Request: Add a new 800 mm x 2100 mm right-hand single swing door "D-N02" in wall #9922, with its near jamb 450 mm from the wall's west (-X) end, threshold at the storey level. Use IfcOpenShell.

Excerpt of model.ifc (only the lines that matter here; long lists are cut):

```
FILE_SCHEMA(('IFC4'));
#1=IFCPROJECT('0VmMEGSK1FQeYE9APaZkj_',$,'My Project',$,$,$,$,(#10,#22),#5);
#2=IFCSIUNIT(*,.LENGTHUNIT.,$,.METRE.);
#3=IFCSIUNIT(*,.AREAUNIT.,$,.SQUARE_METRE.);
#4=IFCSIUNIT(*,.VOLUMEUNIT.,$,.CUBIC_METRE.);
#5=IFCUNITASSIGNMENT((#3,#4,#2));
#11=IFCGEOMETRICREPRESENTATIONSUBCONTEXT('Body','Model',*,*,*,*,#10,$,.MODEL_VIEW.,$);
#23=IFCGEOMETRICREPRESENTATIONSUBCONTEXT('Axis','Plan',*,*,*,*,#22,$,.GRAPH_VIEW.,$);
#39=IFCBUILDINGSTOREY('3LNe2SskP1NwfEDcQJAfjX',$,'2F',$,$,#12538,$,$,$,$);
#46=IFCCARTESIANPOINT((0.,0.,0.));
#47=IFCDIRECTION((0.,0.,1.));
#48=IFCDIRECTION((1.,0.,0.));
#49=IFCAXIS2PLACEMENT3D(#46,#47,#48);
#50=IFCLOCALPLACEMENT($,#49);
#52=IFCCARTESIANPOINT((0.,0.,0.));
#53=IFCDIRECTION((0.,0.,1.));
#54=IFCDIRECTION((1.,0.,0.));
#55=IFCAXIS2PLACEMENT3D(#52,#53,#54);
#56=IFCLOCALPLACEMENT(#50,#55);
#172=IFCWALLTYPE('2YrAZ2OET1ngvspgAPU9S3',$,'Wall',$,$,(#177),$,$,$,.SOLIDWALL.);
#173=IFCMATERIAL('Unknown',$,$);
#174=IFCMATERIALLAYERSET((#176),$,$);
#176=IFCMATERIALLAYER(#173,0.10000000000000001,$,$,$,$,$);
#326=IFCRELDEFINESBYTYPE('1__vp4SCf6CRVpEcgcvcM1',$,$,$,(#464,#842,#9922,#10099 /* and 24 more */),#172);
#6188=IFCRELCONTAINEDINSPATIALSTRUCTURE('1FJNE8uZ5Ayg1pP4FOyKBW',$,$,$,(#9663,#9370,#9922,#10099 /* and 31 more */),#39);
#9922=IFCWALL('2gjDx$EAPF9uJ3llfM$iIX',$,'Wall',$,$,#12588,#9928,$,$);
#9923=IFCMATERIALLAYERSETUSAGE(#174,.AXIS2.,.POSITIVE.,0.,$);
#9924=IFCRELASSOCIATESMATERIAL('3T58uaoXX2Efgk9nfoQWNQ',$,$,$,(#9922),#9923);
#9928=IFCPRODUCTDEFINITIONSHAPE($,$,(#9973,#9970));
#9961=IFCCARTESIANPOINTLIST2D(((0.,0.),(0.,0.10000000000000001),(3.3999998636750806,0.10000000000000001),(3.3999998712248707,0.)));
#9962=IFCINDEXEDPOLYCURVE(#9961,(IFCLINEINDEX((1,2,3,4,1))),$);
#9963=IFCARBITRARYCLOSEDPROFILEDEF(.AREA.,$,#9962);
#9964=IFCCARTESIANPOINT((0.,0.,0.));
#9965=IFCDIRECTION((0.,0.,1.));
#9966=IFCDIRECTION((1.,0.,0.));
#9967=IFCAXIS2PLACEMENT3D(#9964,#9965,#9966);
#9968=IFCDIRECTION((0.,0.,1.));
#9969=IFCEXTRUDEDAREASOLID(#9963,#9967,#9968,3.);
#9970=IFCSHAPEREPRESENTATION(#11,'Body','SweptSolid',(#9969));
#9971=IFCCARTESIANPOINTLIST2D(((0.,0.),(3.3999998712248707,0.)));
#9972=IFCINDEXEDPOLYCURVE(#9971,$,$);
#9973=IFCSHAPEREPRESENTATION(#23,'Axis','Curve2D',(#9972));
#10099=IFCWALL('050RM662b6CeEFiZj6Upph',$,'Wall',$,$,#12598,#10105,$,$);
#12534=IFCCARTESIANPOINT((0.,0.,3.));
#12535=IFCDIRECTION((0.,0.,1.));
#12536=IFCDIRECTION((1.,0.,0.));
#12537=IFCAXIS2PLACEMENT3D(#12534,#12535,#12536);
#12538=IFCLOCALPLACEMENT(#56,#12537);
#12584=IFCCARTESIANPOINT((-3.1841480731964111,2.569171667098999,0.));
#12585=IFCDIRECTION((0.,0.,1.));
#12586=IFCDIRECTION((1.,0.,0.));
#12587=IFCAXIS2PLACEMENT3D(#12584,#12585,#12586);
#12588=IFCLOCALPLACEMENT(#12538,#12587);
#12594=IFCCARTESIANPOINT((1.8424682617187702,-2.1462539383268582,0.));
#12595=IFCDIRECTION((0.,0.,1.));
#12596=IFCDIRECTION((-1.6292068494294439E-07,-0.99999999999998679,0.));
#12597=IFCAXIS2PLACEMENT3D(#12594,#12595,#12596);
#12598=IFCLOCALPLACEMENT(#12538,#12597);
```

```python
import numpy as np
import ifcopenshell
import ifcopenshell.api.feature
import ifcopenshell.api.geometry
import ifcopenshell.api.root
import ifcopenshell.api.spatial
import ifcopenshell.geom
import ifcopenshell.util.element
import ifcopenshell.util.placement
import ifcopenshell.util.representation
import ifcopenshell.util.shape
import ifcopenshell.util.unit

model = ifcopenshell.open("model.ifc")
unit_scale = ifcopenshell.util.unit.calculate_unit_scale(model)
settings = ifcopenshell.geom.settings()


def volume(element):
    """Net volume in cubic metres, openings subtracted."""
    shape = ifcopenshell.geom.create_shape(settings, element)
    return ifcopenshell.util.shape.get_volume(shape.geometry)


wall = model.by_guid("2gjDx$EAPF9uJ3llfM$iIX")
storey = ifcopenshell.util.element.get_container(wall, ifc_class="IfcBuildingStorey")
context = ifcopenshell.util.representation.get_context(model, "Model", "Body", "MODEL_VIEW")
before = volume(wall)

width, height, from_end, sill = 0.8, 2.1, 0.45, 0.0  # metres

# The wall runs along its own X axis, and the end named is its -X end.
wall_shape = ifcopenshell.geom.create_shape(settings, wall)
x, y, z = ifcopenshell.util.shape.get_vertices(wall_shape.geometry).T
start = x.min() + from_end
face, thickness = float(y.min()), float(y.max() - y.min())
wall_matrix = ifcopenshell.util.placement.get_local_placement(wall.ObjectPlacement)
level = ifcopenshell.util.placement.get_local_placement(storey.ObjectPlacement)[2, 3]


def in_wall(x, y):
    """Placement at x, y metres in the wall's axes, at sill height."""
    matrix = wall_matrix.copy()
    matrix[:, 3] = wall_matrix @ np.array([x / unit_scale, y / unit_scale, 0.0, 1.0])
    matrix[2, 3] = level + sill / unit_scale
    return matrix


# Opening: a box that overshoots both wall faces by 50 mm.
opening = ifcopenshell.api.root.create_entity(model, ifc_class="IfcOpeningElement", predefined_type="OPENING")
box = ifcopenshell.api.geometry.add_wall_representation(
    model, context=context, length=width, height=height, thickness=thickness + 0.1
)
ifcopenshell.api.geometry.assign_representation(model, product=opening, representation=box)
ifcopenshell.api.geometry.edit_object_placement(model, product=opening, matrix=in_wall(start, face - 0.05), is_si=False)
ifcopenshell.api.feature.add_feature(model, feature=opening, element=wall)

door = ifcopenshell.api.root.create_entity(model, ifc_class="IfcDoor", name="D-N02", predefined_type="DOOR")
door.OverallWidth, door.OverallHeight = width / unit_scale, height / unit_scale
door.OperationType = "SINGLE_SWING_RIGHT"
body = ifcopenshell.api.geometry.add_door_representation(
    model,
    context=context,
    overall_width=door.OverallWidth,
    overall_height=door.OverallHeight,
    operation_type="SINGLE_SWING_RIGHT",
    lining_properties={"LiningDepth": thickness / unit_scale, "ThresholdDepth": thickness / unit_scale},
)
ifcopenshell.api.geometry.assign_representation(model, product=door, representation=body)
ifcopenshell.api.spatial.assign_container(model, products=[door], relating_structure=storey)
ifcopenshell.api.feature.add_filling(model, opening=opening, element=door)

# The lining spans the wall, so the door starts at the wall face.
ifcopenshell.api.geometry.edit_object_placement(model, product=door, matrix=in_wall(start, face), is_si=False)

after = volume(wall)

print(f"wall volume {before:.3f} -> {after:.3f} m3")

model.write("model_updated.ifc")
```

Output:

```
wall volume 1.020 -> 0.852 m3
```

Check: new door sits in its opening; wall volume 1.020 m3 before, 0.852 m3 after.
